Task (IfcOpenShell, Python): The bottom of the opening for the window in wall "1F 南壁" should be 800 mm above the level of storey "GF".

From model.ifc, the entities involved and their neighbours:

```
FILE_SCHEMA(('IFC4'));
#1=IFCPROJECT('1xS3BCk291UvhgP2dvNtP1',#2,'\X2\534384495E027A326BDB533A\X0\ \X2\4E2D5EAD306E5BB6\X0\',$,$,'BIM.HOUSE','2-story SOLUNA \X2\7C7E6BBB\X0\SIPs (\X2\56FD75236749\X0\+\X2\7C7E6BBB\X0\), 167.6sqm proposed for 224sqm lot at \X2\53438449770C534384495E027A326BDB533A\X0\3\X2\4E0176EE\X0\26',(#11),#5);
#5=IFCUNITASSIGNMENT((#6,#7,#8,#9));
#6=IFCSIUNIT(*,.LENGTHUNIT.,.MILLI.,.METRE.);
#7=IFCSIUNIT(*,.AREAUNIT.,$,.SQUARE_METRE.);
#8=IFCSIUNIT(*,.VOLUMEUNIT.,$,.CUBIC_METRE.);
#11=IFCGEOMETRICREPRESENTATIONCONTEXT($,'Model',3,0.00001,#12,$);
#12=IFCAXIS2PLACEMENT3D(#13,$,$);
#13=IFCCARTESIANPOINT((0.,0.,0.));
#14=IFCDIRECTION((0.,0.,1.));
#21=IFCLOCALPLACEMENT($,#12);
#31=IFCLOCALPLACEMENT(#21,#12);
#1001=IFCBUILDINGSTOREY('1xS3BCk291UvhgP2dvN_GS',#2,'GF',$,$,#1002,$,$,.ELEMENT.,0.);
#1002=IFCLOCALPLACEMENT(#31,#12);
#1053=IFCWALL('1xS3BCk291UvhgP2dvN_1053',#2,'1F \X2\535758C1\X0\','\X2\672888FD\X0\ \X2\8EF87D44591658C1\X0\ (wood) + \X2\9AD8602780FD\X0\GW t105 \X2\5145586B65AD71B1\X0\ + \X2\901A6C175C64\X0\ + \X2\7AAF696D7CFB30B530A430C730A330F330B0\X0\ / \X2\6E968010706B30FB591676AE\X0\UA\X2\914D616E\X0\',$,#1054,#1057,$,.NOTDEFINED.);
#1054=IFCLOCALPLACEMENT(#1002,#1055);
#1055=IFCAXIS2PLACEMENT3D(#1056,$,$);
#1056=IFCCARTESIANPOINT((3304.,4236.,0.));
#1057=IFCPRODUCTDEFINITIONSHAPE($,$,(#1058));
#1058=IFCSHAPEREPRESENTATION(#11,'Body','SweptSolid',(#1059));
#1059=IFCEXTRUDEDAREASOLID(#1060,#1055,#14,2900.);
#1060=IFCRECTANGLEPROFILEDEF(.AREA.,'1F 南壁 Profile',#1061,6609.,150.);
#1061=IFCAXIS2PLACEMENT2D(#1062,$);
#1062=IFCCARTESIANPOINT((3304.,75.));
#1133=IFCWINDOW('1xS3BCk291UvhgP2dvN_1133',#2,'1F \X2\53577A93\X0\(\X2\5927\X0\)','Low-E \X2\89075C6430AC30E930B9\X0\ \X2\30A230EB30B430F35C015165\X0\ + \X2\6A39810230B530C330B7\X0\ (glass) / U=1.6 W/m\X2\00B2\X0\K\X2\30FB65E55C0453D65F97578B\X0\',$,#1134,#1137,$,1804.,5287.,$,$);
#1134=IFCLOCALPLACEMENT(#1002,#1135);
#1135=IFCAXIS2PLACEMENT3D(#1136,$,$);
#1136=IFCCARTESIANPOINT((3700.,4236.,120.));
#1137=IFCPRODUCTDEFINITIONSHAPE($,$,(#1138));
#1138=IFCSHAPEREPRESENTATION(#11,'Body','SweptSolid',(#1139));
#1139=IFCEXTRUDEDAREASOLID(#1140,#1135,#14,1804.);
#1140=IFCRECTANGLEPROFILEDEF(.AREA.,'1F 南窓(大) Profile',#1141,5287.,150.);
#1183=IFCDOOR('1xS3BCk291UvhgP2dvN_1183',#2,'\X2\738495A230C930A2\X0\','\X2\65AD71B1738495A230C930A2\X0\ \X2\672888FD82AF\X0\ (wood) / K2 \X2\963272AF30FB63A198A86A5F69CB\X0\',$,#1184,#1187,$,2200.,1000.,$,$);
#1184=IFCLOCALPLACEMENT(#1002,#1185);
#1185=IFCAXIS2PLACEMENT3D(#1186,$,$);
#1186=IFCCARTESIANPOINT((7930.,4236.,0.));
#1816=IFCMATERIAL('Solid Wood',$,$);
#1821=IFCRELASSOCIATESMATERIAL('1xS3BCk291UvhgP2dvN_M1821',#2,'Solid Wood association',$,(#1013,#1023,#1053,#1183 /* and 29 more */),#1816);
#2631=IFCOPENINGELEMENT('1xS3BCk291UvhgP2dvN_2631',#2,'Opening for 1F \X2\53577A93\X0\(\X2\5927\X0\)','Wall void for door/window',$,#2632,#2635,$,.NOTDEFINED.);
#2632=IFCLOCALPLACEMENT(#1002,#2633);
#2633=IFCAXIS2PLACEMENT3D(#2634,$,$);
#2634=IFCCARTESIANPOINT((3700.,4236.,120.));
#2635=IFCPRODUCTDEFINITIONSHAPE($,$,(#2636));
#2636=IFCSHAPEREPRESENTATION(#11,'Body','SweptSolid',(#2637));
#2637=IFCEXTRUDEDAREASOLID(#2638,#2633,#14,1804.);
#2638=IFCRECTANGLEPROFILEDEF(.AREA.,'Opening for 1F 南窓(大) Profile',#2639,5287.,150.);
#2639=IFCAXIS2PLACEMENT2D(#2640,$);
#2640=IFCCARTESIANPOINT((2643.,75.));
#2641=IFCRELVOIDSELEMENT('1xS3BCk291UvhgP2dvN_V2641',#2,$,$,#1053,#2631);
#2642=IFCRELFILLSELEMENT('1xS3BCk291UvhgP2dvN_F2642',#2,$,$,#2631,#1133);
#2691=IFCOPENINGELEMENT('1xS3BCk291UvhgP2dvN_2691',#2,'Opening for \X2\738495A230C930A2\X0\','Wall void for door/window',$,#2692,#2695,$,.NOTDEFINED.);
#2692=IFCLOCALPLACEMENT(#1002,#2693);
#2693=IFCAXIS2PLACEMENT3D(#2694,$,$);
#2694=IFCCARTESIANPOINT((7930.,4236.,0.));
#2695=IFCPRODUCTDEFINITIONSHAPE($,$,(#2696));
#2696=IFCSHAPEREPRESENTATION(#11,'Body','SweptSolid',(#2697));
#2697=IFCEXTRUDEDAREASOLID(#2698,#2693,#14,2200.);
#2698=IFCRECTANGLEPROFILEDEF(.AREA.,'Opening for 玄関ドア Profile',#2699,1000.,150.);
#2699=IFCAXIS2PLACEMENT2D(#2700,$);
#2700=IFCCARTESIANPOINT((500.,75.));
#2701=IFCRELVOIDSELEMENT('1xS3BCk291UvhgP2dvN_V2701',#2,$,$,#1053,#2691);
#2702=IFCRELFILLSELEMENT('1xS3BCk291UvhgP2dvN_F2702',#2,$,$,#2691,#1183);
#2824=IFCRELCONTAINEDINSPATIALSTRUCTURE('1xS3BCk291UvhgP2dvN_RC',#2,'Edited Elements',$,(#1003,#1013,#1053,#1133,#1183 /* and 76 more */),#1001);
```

```python
import numpy as np
import ifcopenshell
import ifcopenshell.api.geometry
import ifcopenshell.geom
import ifcopenshell.util.element
import ifcopenshell.util.placement
import ifcopenshell.util.shape
import ifcopenshell.util.unit

model = ifcopenshell.open("model.ifc")
unit_scale = ifcopenshell.util.unit.calculate_unit_scale(model)

window = model.by_guid("1xS3BCk291UvhgP2dvN_1133")
opening = window.FillsVoids[0].RelatingOpeningElement
storey = ifcopenshell.util.element.get_container(window, ifc_class="IfcBuildingStorey")
level = ifcopenshell.util.placement.get_local_placement(storey.ObjectPlacement)[2, 3]

# The opening's origin need not be at the sill, so measure its lowest point.
shape = ifcopenshell.geom.create_shape(ifcopenshell.geom.settings(), opening)
bottom = ifcopenshell.util.shape.get_shape_bottom_elevation(shape, shape.geometry) / unit_scale
dz = level + 800.0 - bottom

shift = np.array([0.0, 0.0, dz])
# The window is not placed relative to its opening, so move both.
for product in (opening, window):
    matrix = ifcopenshell.util.placement.get_local_placement(product.ObjectPlacement)
    matrix[:3, 3] += shift
    ifcopenshell.api.geometry.edit_object_placement(model, product=product, matrix=matrix, is_si=False)

print(f"moved by {dz * unit_scale:+.3f} m")

model.write("model-out.ifc")
```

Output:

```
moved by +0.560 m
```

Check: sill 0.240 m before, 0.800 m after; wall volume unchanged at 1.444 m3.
